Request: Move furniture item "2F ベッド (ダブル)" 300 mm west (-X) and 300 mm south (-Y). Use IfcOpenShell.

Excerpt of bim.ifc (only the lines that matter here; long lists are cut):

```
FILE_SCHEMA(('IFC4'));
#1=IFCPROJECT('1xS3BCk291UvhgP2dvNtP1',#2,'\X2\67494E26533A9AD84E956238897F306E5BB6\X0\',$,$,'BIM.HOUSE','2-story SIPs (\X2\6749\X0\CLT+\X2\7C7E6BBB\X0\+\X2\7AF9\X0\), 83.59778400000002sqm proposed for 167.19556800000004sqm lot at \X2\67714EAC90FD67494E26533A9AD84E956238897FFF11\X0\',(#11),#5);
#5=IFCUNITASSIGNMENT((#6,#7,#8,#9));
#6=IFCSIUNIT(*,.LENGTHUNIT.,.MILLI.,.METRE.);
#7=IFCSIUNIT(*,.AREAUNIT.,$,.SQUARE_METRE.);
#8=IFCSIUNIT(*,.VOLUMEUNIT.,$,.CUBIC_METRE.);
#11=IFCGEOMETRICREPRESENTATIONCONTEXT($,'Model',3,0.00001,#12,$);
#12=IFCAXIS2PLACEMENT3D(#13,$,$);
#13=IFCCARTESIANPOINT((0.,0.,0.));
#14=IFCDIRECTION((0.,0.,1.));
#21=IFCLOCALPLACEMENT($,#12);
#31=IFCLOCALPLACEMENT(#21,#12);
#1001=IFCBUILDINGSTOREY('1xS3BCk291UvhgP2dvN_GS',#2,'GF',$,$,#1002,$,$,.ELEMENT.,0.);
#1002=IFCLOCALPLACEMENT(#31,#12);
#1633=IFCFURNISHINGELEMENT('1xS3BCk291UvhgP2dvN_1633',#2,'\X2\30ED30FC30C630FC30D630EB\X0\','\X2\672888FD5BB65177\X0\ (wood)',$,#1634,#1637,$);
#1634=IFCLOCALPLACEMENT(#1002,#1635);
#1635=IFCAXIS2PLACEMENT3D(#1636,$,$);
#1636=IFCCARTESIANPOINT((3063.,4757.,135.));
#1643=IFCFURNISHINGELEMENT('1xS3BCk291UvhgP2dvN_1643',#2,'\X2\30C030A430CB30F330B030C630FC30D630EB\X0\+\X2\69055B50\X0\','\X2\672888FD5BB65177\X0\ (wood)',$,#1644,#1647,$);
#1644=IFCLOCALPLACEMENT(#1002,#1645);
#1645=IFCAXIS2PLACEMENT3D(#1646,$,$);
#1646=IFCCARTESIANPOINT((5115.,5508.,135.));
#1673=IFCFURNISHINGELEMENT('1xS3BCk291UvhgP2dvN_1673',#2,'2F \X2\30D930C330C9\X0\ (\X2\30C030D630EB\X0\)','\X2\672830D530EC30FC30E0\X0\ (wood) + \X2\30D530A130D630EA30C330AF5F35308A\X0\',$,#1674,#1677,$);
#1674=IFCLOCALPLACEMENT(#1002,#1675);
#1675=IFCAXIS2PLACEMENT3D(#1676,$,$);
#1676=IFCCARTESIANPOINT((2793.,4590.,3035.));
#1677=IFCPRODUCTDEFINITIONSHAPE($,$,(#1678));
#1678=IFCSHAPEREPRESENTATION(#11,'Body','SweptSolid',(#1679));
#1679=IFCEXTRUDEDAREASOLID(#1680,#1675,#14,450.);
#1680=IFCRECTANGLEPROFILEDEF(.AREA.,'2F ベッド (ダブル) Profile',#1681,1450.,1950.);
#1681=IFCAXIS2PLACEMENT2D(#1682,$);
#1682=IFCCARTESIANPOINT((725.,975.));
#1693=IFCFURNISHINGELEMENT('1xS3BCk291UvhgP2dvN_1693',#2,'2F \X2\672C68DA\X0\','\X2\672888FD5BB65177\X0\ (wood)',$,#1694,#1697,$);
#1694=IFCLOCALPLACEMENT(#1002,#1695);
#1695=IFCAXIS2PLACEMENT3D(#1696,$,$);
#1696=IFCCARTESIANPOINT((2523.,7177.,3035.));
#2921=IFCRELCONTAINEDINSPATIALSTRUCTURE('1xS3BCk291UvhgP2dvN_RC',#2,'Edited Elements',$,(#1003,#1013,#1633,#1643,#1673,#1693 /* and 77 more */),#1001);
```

```python
import ifcopenshell
import ifcopenshell.api.geometry
import ifcopenshell.util.placement
import ifcopenshell.util.unit

model = ifcopenshell.open("bim.ifc")
unit_scale = ifcopenshell.util.unit.calculate_unit_scale(model)

item = model.by_guid("1xS3BCk291UvhgP2dvN_1673")
matrix = ifcopenshell.util.placement.get_local_placement(item.ObjectPlacement)
matrix[0, 3] -= 0.3 / unit_scale
matrix[1, 3] -= 0.3 / unit_scale
ifcopenshell.api.geometry.edit_object_placement(model, product=item, matrix=matrix, is_si=False)

print(ifcopenshell.util.placement.get_local_placement(item.ObjectPlacement).round(3) + 0.0)

model.write("bim_edited.ifc")
```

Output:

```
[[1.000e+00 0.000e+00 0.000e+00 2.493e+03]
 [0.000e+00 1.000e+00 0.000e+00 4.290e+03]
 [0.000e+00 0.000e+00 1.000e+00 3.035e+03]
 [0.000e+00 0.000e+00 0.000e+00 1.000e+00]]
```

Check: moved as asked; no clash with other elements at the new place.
